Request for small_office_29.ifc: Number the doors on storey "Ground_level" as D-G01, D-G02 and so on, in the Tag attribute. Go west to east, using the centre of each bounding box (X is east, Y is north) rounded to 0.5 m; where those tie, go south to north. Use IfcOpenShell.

First a look at what the model holds.

```python
import ifcopenshell
import ifcopenshell.util.element
import ifcopenshell.util.placement

model = ifcopenshell.open("small_office_29.ifc")
print(model.schema)
storey = next(s for s in model.by_type("IfcBuildingStorey") if s.Name == "Ground_level")
doors = [e for e in ifcopenshell.util.element.get_decomposition(storey) if e.is_a("IfcDoor")]
for e in sorted(doors, key=lambda e: e.id()):
    origin = ifcopenshell.util.placement.get_local_placement(e.ObjectPlacement)[:3, 3]
    print(e.id(), e.Tag, e.Name, origin.round(2) + 0.0, sep=" | ")
```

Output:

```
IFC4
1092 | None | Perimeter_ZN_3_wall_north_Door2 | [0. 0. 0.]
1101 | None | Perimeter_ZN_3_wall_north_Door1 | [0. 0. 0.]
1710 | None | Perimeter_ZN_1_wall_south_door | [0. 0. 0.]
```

```python
import ifcopenshell
import ifcopenshell.geom
import ifcopenshell.util.element
import ifcopenshell.util.shape

model = ifcopenshell.open("small_office_29.ifc")
settings = ifcopenshell.geom.settings()
settings.set("use-world-coords", True)


def centre(element):
    shape = ifcopenshell.geom.create_shape(settings, element)
    return ifcopenshell.util.shape.get_bbox_centroid(shape.geometry)


storey = next(s for s in model.by_type("IfcBuildingStorey") if s.Name == "Ground_level")
doors = [e for e in ifcopenshell.util.element.get_decomposition(storey) if e.is_a("IfcDoor")]

# Insertion points can sit at a corner or the storey origin, so sort by the geometry (in metres).
centres = {e: centre(e) for e in doors}
doors.sort(key=lambda e: (round(centres[e][0] / 0.5), centres[e][1]))

for i, e in enumerate(doors, start=1):
    number = f"D-G{i:02d}"
    e.Tag = number
    print(e.id(), number)

model.write("small_office_29-out.ifc")
```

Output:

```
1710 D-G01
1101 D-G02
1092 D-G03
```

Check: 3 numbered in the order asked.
